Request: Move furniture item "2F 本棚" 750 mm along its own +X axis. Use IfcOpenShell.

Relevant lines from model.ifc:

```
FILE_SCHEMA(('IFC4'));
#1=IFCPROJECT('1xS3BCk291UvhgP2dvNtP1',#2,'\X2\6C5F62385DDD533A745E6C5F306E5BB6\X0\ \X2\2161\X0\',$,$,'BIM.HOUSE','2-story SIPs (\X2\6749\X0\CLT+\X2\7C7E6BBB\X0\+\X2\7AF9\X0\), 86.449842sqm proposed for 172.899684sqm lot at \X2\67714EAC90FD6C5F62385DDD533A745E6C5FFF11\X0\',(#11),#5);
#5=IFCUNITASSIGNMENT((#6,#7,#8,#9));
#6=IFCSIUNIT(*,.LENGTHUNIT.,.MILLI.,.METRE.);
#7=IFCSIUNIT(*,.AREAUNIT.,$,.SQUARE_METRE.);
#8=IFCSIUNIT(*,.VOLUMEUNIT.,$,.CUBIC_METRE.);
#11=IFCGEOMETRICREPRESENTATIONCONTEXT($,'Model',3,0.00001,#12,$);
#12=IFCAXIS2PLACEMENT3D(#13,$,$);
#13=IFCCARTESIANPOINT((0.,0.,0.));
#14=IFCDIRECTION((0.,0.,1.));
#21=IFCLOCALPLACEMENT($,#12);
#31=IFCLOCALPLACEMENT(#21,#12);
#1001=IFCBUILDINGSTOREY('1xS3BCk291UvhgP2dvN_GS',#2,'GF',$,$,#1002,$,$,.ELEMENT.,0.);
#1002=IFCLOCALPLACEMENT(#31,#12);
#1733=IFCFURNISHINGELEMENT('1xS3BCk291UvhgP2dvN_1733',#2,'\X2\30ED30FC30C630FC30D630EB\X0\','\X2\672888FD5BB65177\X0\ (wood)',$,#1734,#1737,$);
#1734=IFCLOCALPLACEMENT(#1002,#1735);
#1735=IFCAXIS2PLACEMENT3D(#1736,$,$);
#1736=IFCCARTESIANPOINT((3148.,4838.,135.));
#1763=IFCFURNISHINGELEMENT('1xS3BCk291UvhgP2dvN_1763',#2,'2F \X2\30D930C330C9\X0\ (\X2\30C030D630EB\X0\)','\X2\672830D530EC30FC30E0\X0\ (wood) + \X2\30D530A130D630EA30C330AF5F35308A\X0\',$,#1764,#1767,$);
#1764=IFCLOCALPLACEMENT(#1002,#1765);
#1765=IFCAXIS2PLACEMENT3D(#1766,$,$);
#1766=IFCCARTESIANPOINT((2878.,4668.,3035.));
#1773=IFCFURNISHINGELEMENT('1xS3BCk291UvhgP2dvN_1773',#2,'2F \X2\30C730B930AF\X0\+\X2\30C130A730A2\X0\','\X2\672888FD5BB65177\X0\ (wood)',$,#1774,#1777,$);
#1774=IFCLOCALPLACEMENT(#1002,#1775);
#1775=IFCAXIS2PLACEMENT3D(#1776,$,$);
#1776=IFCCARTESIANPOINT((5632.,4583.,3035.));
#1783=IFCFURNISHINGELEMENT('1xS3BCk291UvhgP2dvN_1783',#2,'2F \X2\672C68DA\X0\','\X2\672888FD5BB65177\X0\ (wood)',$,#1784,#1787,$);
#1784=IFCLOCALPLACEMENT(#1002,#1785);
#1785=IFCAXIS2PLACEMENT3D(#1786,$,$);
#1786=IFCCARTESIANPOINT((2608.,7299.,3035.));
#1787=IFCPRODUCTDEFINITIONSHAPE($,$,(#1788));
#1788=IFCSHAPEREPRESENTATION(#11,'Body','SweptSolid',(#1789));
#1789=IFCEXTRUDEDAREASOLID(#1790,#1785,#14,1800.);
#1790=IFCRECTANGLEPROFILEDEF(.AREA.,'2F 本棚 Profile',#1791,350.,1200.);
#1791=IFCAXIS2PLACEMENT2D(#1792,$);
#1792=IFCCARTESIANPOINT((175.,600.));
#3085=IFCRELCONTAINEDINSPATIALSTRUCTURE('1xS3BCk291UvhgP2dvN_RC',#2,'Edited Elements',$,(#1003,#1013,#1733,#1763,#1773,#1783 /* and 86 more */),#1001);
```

```python
import ifcopenshell
import ifcopenshell.api.geometry
import ifcopenshell.util.placement
import ifcopenshell.util.unit

model = ifcopenshell.open("model.ifc")
unit_scale = ifcopenshell.util.unit.calculate_unit_scale(model)

item = model.by_guid("1xS3BCk291UvhgP2dvN_1783")
matrix = ifcopenshell.util.placement.get_local_placement(item.ObjectPlacement)
matrix[:3, 3] += matrix[:3, 0] * 0.75 / unit_scale
ifcopenshell.api.geometry.edit_object_placement(model, product=item, matrix=matrix, is_si=False)

print(ifcopenshell.util.placement.get_local_placement(item.ObjectPlacement).round(3) + 0.0)

model.write("model_rev.ifc")
```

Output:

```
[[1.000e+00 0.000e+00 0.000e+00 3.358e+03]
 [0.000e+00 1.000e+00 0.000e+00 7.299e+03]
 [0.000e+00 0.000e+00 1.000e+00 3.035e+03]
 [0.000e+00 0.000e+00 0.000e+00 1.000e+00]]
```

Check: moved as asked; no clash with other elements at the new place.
